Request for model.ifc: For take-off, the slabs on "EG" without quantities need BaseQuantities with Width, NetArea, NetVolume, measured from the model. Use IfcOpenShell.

First a look at what the model holds.

```python
import ifcopenshell
import ifcopenshell.util.element
import ifcopenshell.util.unit

model = ifcopenshell.open("model.ifc")
print(model.schema)
for unit_type in ("LENGTHUNIT", "AREAUNIT", "VOLUMEUNIT"):
    print(unit_type, ifcopenshell.util.unit.calculate_unit_scale(model, unit_type))
storey = next(s for s in model.by_type("IfcBuildingStorey") if s.Name == "EG")
slabs = [e for e in ifcopenshell.util.element.get_decomposition(storey) if e.is_a("IfcSlab")]
for e in sorted(slabs, key=lambda e: e.id()):
    print(e.id(), e.is_a(), e.Name, list(ifcopenshell.util.element.get_psets(e, qtos_only=True)), sep=" | ")
```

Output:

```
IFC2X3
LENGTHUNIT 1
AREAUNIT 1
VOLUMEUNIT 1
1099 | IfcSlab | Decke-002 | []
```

```python
import ifcopenshell
import ifcopenshell.api.pset
import ifcopenshell.geom
import ifcopenshell.util.element
import ifcopenshell.util.shape
import ifcopenshell.util.unit

model = ifcopenshell.open("model.ifc")
unit_scale = ifcopenshell.util.unit.calculate_unit_scale(model)
area_scale = ifcopenshell.util.unit.calculate_unit_scale(model, "AREAUNIT")
volume_scale = ifcopenshell.util.unit.calculate_unit_scale(model, "VOLUMEUNIT")
settings = ifcopenshell.geom.settings()

storey = next(s for s in model.by_type("IfcBuildingStorey") if s.Name == "EG")
slabs = [e for e in ifcopenshell.util.element.get_decomposition(storey) if e.is_a("IfcSlab")]

for e in sorted(slabs, key=lambda e: e.id()):
    if ifcopenshell.util.element.get_psets(e, qtos_only=True, should_inherit=False):
        continue
    # Geometry comes back in metres, in the element's own axes.
    shape = ifcopenshell.geom.create_shape(settings, e)
    values = {
        "Width": ifcopenshell.util.shape.get_z(shape.geometry) / unit_scale,
        "NetArea": ifcopenshell.util.shape.get_footprint_area(shape.geometry) / area_scale,
        "NetVolume": ifcopenshell.util.shape.get_volume(shape.geometry) / volume_scale,
    }
    qto = ifcopenshell.api.pset.add_qto(model, product=e, name="BaseQuantities")
    ifcopenshell.api.pset.edit_qto(model, qto=qto, properties=values)
    print(e.id(), {k: round(v, 3) for k, v in values.items()})

model.write("model_updated.ifc")
```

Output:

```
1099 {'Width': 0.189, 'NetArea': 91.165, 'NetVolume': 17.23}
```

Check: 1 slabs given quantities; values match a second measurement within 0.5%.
